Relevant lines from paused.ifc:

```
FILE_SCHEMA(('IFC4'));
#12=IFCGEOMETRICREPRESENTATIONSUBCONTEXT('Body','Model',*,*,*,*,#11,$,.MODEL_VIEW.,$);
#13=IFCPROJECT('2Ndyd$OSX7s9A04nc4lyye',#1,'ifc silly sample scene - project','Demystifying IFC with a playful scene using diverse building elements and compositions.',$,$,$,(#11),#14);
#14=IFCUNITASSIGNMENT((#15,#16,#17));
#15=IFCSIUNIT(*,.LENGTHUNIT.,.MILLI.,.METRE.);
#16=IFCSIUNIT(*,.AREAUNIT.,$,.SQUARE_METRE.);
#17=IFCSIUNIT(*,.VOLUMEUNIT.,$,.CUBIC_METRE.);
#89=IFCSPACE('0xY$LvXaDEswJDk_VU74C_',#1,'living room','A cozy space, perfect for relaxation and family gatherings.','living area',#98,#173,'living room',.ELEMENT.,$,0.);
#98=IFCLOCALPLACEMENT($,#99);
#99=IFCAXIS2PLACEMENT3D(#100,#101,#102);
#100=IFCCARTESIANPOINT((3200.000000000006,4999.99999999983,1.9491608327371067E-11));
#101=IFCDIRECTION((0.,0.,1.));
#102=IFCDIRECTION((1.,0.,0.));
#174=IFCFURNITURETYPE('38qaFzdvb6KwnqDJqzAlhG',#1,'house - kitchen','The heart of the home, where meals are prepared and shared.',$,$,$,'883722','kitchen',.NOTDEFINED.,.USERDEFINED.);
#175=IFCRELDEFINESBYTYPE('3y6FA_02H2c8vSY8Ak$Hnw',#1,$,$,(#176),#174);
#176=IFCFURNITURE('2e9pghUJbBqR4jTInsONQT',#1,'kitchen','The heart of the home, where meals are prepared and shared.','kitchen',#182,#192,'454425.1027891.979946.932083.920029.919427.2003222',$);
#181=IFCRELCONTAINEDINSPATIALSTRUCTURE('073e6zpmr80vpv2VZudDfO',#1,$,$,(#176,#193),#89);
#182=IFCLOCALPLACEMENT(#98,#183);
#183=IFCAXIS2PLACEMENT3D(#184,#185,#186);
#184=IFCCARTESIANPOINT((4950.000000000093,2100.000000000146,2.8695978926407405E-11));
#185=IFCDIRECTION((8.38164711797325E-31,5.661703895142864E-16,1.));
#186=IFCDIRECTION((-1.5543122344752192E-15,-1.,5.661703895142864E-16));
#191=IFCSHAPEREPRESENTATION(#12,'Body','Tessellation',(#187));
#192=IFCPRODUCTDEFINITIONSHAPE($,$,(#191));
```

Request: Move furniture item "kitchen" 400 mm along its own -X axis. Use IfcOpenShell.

```python
import ifcopenshell
import ifcopenshell.api.geometry
import ifcopenshell.util.placement
import ifcopenshell.util.unit

model = ifcopenshell.open("paused.ifc")
unit_scale = ifcopenshell.util.unit.calculate_unit_scale(model)

item = model.by_id(176)
matrix = ifcopenshell.util.placement.get_local_placement(item.ObjectPlacement)
matrix[:3, 3] -= matrix[:3, 0] * 0.4 / unit_scale
ifcopenshell.api.geometry.edit_object_placement(model, product=item, matrix=matrix, is_si=False)

print(ifcopenshell.util.placement.get_local_placement(item.ObjectPlacement).round(3) + 0.0)

model.write("paused_v2.ifc")
```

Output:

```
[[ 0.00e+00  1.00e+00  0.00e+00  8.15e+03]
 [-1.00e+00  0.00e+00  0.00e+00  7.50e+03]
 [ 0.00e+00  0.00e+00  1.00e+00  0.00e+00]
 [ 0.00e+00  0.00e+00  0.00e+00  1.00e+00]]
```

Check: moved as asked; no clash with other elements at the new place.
